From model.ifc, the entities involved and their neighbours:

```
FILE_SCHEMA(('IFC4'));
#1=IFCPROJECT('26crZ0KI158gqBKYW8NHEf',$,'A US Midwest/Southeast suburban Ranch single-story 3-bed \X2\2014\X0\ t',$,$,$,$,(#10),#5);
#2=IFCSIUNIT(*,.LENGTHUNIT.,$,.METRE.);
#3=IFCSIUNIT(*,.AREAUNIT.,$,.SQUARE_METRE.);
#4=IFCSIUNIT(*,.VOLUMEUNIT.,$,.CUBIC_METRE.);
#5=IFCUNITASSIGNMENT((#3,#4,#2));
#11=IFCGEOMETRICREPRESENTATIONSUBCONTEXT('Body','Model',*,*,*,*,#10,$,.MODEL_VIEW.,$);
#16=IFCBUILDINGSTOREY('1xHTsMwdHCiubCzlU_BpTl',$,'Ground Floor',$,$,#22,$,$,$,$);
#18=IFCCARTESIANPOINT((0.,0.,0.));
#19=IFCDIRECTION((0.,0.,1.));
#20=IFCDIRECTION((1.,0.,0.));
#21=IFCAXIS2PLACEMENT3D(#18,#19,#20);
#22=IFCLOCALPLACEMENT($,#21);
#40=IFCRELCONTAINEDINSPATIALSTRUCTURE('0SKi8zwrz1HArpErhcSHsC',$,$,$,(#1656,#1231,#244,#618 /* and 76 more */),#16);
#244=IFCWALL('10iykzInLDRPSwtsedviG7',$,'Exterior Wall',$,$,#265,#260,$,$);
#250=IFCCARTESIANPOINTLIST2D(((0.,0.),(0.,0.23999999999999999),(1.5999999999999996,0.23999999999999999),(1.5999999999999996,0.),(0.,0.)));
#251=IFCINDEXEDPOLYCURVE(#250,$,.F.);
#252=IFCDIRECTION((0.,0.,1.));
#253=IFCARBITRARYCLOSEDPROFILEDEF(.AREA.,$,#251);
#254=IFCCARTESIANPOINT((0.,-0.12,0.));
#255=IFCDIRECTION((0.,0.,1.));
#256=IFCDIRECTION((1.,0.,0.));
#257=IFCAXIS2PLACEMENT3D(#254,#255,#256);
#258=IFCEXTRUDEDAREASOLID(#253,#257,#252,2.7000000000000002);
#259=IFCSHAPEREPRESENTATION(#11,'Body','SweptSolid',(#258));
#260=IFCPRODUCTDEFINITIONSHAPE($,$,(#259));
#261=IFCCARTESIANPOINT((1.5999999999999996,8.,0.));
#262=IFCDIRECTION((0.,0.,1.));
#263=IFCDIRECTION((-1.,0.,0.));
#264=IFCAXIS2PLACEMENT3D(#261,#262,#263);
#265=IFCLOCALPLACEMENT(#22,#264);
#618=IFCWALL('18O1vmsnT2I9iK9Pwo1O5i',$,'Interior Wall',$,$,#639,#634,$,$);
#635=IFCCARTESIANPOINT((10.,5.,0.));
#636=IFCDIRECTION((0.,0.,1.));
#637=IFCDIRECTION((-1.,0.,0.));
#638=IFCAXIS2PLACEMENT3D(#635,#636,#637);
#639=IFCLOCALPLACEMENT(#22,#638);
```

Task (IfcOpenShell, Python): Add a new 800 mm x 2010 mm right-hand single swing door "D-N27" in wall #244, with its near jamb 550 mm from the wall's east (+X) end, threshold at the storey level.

```python
import numpy as np
import ifcopenshell
import ifcopenshell.api.feature
import ifcopenshell.api.geometry
import ifcopenshell.api.root
import ifcopenshell.api.spatial
import ifcopenshell.geom
import ifcopenshell.util.element
import ifcopenshell.util.placement
import ifcopenshell.util.representation
import ifcopenshell.util.shape
import ifcopenshell.util.unit

model = ifcopenshell.open("model.ifc")
unit_scale = ifcopenshell.util.unit.calculate_unit_scale(model)
settings = ifcopenshell.geom.settings()


def volume(element):
    """Net volume in cubic metres, openings subtracted."""
    shape = ifcopenshell.geom.create_shape(settings, element)
    return ifcopenshell.util.shape.get_volume(shape.geometry)


wall = model.by_guid("10iykzInLDRPSwtsedviG7")
storey = ifcopenshell.util.element.get_container(wall, ifc_class="IfcBuildingStorey")
context = ifcopenshell.util.representation.get_context(model, "Model", "Body", "MODEL_VIEW")
before = volume(wall)

width, height, from_end, sill = 0.8, 2.01, 0.55, 0.0  # metres

# The wall runs along its own X axis, and the end named is its -X end.
wall_shape = ifcopenshell.geom.create_shape(settings, wall)
x, y, z = ifcopenshell.util.shape.get_vertices(wall_shape.geometry).T
start = x.min() + from_end
face, thickness = float(y.min()), float(y.max() - y.min())
wall_matrix = ifcopenshell.util.placement.get_local_placement(wall.ObjectPlacement)
level = ifcopenshell.util.placement.get_local_placement(storey.ObjectPlacement)[2, 3]


def in_wall(x, y):
    """Placement at x, y metres in the wall's axes, at sill height."""
    matrix = wall_matrix.copy()
    matrix[:, 3] = wall_matrix @ np.array([x / unit_scale, y / unit_scale, 0.0, 1.0])
    matrix[2, 3] = level + sill / unit_scale
    return matrix


# Opening: a box that overshoots both wall faces by 50 mm.
opening = ifcopenshell.api.root.create_entity(model, ifc_class="IfcOpeningElement", predefined_type="OPENING")
box = ifcopenshell.api.geometry.add_wall_representation(
    model, context=context, length=width, height=height, thickness=thickness + 0.1
)
ifcopenshell.api.geometry.assign_representation(model, product=opening, representation=box)
ifcopenshell.api.geometry.edit_object_placement(model, product=opening, matrix=in_wall(start, face - 0.05), is_si=False)
ifcopenshell.api.feature.add_feature(model, feature=opening, element=wall)

door = ifcopenshell.api.root.create_entity(model, ifc_class="IfcDoor", name="D-N27", predefined_type="DOOR")
door.OverallWidth, door.OverallHeight = width / unit_scale, height / unit_scale
door.OperationType = "SINGLE_SWING_RIGHT"
body = ifcopenshell.api.geometry.add_door_representation(
    model,
    context=context,
    overall_width=door.OverallWidth,
    overall_height=door.OverallHeight,
    operation_type="SINGLE_SWING_RIGHT",
    lining_properties={"LiningDepth": thickness / unit_scale, "ThresholdDepth": thickness / unit_scale},
)
ifcopenshell.api.geometry.assign_representation(model, product=door, representation=body)
ifcopenshell.api.spatial.assign_container(model, products=[door], relating_structure=storey)
ifcopenshell.api.feature.add_filling(model, opening=opening, element=door)

# The lining spans the wall, so the door starts at the wall face.
ifcopenshell.api.geometry.edit_object_placement(model, product=door, matrix=in_wall(start, face), is_si=False)

after = volume(wall)

print(f"wall volume {before:.3f} -> {after:.3f} m3")

model.write("model_v2.ifc")
```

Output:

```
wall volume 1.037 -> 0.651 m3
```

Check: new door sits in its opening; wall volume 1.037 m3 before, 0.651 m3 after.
